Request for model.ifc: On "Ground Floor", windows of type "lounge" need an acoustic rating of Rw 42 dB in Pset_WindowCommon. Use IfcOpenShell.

First a look at what the model holds.

```python
import ifcopenshell
import ifcopenshell.util.element

model = ifcopenshell.open("model.ifc")
print(model.schema)
storey = next(s for s in model.by_type("IfcBuildingStorey") if s.Name == "Ground Floor")
windows = [e for e in ifcopenshell.util.element.get_decomposition(storey) if e.is_a("IfcWindow")]
seen = {}
for e in windows:
    element_type = ifcopenshell.util.element.get_type(e)
    key = (element_type.Name if element_type != e and element_type else None, ifcopenshell.util.element.get_pset(e, "Pset_WindowCommon", "AcousticRating"))
    seen[key] = seen.get(key, 0) + 1
for (name, value), count in sorted(seen.items(), key=str):
    print(count, "x", name, "|", value)
```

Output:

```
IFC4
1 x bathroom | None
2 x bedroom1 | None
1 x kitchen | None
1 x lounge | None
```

```python
import ifcopenshell
import ifcopenshell.api.pset
import ifcopenshell.util.element

model = ifcopenshell.open("model.ifc")

storey = next(s for s in model.by_type("IfcBuildingStorey") if s.Name == "Ground Floor")
windows = [e for e in ifcopenshell.util.element.get_decomposition(storey) if e.is_a("IfcWindow")]

count = 0
for e in windows:
    element_type = ifcopenshell.util.element.get_type(e)
    if element_type in (None, e) or element_type.Name != "lounge":
        continue
    # add_pset returns the element's existing set when there is one.
    pset = ifcopenshell.api.pset.add_pset(model, product=e, name="Pset_WindowCommon")
    ifcopenshell.api.pset.edit_pset(model, pset=pset, properties={"AcousticRating": "Rw 42 dB"})
    count += 1

print(count, "windows updated")

model.write("model_updated.ifc")
```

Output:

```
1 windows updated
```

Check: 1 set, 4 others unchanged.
